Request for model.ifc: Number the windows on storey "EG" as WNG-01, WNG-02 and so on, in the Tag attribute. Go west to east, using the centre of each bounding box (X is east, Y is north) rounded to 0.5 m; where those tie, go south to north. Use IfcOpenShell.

First a look at what the model holds.

```python
import ifcopenshell
import ifcopenshell.util.element
import ifcopenshell.util.placement

model = ifcopenshell.open("model.ifc")
print(model.schema)
storey = next(s for s in model.by_type("IfcBuildingStorey") if s.Name == "EG")
windows = [e for e in ifcopenshell.util.element.get_decomposition(storey) if e.is_a("IfcWindow")]
for e in sorted(windows, key=lambda e: e.id()):
    origin = ifcopenshell.util.placement.get_local_placement(e.ObjectPlacement)[:3, 3]
    print(e.id(), e.Tag, e.Name, origin.round(2) + 0.0, sep=" | ")
```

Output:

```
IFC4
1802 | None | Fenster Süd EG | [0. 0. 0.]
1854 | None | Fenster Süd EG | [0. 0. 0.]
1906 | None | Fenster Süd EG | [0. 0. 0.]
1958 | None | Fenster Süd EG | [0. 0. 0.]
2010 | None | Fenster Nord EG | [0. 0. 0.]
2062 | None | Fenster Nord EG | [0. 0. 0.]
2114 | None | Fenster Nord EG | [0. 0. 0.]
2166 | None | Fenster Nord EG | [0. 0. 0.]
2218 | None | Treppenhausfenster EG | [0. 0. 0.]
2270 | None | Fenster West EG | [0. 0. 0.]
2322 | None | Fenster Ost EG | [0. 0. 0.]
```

```python
import ifcopenshell
import ifcopenshell.geom
import ifcopenshell.util.element
import ifcopenshell.util.shape

model = ifcopenshell.open("model.ifc")
settings = ifcopenshell.geom.settings()
settings.set("use-world-coords", True)


def centre(element):
    shape = ifcopenshell.geom.create_shape(settings, element)
    return ifcopenshell.util.shape.get_bbox_centroid(shape.geometry)


storey = next(s for s in model.by_type("IfcBuildingStorey") if s.Name == "EG")
windows = [e for e in ifcopenshell.util.element.get_decomposition(storey) if e.is_a("IfcWindow")]

# Insertion points can sit at a corner or the storey origin, so sort by the geometry (in metres).
centres = {e: centre(e) for e in windows}
windows.sort(key=lambda e: (round(centres[e][0] / 0.5), centres[e][1]))

for i, e in enumerate(windows, start=1):
    number = f"WNG-{i:02d}"
    e.Tag = number
    print(e.id(), number)

model.write("model_rev.ifc")
```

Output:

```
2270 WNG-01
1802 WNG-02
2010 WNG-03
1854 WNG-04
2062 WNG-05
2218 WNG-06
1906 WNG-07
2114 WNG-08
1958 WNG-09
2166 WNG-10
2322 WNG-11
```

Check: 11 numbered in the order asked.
